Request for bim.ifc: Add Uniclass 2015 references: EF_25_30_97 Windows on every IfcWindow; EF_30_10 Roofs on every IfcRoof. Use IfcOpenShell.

First a look at what the model holds.

```python
import ifcopenshell

model = ifcopenshell.open("bim.ifc")
print(model.schema)
print("classifications:", [c.Name for c in model.by_type("IfcClassification")])
for ifc_class in ("IfcDoor", "IfcRoof", "IfcStair", "IfcWall", "IfcWindow"):
    print(ifc_class, len(model.by_type(ifc_class)))
```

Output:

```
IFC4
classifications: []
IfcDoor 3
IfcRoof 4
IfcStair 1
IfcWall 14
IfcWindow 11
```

```python
import ifcopenshell
import ifcopenshell.api.classification

model = ifcopenshell.open("bim.ifc")

system = ifcopenshell.api.classification.add_classification(model, classification="Uniclass 2015")

codes = {
    "IfcWindow": ("EF_25_30_97", "Windows"),
    "IfcRoof": ("EF_30_10", "Roofs"),
}
for ifc_class, (code, name) in codes.items():
    products = model.by_type(ifc_class)
    ifcopenshell.api.classification.add_reference(
        model, products=products, classification=system, identification=code, name=name
    )
    print(code, len(products))

model.write("bim_v2.ifc")
```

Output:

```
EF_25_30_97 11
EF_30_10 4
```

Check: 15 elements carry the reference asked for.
